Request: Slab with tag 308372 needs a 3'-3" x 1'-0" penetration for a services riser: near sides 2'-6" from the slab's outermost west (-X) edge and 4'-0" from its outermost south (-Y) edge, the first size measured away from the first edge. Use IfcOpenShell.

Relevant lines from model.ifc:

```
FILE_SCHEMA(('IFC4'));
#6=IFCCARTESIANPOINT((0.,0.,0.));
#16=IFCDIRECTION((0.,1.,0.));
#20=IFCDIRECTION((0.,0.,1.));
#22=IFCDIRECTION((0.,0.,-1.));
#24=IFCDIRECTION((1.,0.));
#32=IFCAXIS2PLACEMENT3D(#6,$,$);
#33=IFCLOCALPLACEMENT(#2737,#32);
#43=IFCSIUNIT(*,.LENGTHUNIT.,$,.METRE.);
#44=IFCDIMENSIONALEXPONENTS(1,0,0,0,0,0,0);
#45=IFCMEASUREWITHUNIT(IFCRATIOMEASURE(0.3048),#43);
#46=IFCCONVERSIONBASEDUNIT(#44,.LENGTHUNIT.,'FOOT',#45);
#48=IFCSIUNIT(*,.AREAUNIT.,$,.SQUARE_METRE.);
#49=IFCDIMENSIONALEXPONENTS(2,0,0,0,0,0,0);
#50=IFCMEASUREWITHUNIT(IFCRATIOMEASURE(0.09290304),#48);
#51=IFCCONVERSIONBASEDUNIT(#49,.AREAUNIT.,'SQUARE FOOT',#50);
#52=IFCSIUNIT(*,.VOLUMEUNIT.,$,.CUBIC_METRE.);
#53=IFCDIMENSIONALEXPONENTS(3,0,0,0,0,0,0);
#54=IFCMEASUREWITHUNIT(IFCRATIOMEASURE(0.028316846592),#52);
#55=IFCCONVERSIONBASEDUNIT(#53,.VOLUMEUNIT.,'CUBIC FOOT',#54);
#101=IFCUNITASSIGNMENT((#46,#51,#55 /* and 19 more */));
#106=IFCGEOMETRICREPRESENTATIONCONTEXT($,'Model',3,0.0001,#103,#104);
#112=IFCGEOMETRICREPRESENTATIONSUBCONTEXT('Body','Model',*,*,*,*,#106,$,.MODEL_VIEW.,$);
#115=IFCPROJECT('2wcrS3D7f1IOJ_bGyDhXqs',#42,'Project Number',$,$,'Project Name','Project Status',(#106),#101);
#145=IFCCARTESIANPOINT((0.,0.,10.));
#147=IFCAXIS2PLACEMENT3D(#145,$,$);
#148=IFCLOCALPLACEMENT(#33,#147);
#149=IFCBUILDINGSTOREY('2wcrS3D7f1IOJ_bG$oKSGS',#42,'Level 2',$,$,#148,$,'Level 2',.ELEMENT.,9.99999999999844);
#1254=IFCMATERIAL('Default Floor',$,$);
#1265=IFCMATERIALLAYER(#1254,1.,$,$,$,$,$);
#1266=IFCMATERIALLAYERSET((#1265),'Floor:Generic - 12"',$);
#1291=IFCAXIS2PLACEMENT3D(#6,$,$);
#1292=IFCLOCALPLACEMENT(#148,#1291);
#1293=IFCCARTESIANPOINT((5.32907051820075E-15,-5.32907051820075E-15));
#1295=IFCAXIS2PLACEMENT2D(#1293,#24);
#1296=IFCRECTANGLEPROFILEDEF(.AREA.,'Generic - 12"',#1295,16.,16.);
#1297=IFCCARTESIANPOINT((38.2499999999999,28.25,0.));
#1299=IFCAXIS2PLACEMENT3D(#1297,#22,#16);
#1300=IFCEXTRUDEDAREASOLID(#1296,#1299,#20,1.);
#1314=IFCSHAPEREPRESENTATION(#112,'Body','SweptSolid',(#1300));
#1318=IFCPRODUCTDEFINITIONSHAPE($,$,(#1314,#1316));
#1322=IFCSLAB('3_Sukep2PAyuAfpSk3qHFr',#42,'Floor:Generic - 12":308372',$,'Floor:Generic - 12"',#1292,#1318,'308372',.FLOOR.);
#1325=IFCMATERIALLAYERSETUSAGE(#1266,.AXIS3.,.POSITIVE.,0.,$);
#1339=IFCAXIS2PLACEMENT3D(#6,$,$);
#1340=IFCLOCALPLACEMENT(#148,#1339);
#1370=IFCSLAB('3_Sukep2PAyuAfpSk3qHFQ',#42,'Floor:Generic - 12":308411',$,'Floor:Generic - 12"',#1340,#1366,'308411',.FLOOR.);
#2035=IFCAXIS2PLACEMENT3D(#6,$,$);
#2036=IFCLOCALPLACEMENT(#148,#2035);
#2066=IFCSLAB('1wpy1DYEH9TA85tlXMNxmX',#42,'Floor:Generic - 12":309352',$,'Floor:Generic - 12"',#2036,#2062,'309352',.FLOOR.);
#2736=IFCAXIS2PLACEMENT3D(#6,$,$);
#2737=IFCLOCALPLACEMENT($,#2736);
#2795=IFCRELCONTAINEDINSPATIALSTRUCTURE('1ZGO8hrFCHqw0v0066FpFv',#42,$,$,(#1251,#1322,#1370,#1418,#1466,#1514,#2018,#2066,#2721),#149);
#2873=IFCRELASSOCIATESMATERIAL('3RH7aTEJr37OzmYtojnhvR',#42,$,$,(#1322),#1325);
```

```python
import numpy as np
import ifcopenshell
import ifcopenshell.api.feature
import ifcopenshell.api.geometry
import ifcopenshell.api.root
import ifcopenshell.geom
import ifcopenshell.util.placement
import ifcopenshell.util.representation
import ifcopenshell.util.shape
import ifcopenshell.util.unit

model = ifcopenshell.open("model.ifc")
unit_scale = ifcopenshell.util.unit.calculate_unit_scale(model)
settings = ifcopenshell.geom.settings()


def volume(element):
    """Net volume in cubic metres, openings subtracted."""
    shape = ifcopenshell.geom.create_shape(settings, element)
    return ifcopenshell.util.shape.get_volume(shape.geometry)


slab = model.by_id(1322)
before = volume(slab)

# Extent in the slab's own axes, in metres. The edges named are its -X and -Y sides.
slab_shape = ifcopenshell.geom.create_shape(settings, slab)
vertices = ifcopenshell.util.shape.get_vertices(slab_shape.geometry)
x_min, y_min, bottom = vertices.min(axis=0)
top = vertices[:, 2].max()

opening = ifcopenshell.api.root.create_entity(model, ifc_class="IfcOpeningElement", name="Services riser opening", predefined_type="OPENING")
context = ifcopenshell.util.representation.get_context(model, "Model", "Body", "MODEL_VIEW")
width, depth = 0.9906, 0.3048
outline = [(0.0, 0.0), (width, 0.0), (width, depth), (0.0, depth), (0.0, 0.0)]
# Overshoot both faces by 50 mm so the cut is clean.
shape = ifcopenshell.api.geometry.add_slab_representation(
    model, context=context, depth=top - bottom + 0.1, polyline=outline
)
ifcopenshell.api.geometry.assign_representation(model, product=opening, representation=shape)

matrix = ifcopenshell.util.placement.get_local_placement(slab.ObjectPlacement)
matrix[:, 3] = matrix @ np.append(np.array([x_min + 0.762, y_min + 1.2192, bottom - 0.05]) / unit_scale, 1.0)
ifcopenshell.api.geometry.edit_object_placement(model, product=opening, matrix=matrix, is_si=False)
ifcopenshell.api.feature.add_feature(model, feature=opening, element=slab)

after = volume(slab)

print(f"slab volume {before:.3f} -> {after:.3f} m3")

model.write("model-out.ifc")
```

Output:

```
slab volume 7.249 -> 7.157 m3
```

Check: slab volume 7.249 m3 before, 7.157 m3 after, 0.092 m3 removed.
